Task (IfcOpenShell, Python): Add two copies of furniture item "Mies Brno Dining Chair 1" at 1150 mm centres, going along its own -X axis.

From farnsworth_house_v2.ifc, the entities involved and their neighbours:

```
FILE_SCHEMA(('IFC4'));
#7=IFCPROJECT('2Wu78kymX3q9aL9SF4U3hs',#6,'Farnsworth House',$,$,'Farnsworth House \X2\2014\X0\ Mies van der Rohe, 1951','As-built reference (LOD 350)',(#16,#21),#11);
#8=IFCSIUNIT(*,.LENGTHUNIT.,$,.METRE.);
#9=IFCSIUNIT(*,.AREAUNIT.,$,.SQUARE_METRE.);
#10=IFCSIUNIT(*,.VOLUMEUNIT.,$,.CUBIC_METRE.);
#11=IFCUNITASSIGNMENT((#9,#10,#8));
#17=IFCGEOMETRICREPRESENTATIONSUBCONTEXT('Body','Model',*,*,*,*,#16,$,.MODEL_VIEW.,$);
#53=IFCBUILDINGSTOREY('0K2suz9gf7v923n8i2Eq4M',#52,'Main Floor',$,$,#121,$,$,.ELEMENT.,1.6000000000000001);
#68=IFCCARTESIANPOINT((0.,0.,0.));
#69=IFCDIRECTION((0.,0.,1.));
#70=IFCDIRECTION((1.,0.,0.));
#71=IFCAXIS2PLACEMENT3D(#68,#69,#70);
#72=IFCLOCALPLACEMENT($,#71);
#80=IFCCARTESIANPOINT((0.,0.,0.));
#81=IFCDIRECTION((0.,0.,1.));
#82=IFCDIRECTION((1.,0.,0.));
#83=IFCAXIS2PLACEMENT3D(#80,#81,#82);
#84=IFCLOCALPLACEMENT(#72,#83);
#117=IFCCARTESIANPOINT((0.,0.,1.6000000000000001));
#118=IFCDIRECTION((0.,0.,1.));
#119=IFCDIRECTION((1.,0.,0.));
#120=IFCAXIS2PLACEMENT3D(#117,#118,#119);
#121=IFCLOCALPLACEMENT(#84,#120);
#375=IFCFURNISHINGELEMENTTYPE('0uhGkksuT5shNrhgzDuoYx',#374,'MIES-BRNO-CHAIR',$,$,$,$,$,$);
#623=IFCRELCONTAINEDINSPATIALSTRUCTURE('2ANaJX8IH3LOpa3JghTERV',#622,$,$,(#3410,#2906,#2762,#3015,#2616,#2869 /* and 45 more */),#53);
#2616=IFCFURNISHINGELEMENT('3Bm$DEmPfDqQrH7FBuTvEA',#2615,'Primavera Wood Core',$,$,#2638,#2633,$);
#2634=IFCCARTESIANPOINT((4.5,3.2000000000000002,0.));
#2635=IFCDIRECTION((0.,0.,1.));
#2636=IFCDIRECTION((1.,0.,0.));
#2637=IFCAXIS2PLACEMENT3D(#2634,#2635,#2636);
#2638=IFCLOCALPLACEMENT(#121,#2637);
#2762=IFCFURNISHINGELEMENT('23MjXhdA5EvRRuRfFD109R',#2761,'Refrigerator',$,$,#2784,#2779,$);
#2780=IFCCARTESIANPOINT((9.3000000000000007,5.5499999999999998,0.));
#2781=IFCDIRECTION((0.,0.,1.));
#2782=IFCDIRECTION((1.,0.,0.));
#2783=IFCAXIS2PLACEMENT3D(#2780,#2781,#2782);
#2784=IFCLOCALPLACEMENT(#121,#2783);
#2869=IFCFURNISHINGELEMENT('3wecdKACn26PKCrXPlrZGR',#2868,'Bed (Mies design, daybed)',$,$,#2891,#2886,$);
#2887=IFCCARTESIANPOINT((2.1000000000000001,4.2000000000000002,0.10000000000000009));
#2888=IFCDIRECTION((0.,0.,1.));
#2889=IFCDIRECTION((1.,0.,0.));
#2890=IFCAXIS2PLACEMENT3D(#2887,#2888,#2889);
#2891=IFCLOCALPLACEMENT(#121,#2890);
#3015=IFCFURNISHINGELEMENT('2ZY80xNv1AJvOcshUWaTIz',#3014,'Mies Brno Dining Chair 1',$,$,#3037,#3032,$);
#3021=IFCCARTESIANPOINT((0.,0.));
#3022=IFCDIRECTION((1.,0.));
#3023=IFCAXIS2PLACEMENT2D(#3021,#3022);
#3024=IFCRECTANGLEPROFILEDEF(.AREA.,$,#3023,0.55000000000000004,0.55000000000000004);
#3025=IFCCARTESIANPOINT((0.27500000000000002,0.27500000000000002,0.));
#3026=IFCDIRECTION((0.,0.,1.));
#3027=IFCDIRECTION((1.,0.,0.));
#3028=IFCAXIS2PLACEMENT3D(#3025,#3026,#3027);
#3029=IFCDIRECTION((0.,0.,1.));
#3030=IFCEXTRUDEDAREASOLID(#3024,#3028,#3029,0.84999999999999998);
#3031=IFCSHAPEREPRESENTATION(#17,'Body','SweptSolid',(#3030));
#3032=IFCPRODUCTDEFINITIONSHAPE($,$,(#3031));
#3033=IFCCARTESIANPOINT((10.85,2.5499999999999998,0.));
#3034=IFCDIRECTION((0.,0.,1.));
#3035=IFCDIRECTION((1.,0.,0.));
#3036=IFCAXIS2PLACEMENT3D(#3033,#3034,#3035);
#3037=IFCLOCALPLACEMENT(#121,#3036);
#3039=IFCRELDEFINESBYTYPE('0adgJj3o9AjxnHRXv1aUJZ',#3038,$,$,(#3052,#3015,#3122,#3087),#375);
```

```python
import ifcopenshell
import ifcopenshell.api.geometry
import ifcopenshell.api.root
import ifcopenshell.util.element
import ifcopenshell.util.placement
import ifcopenshell.util.unit

model = ifcopenshell.open("farnsworth_house_v2.ifc")
unit_scale = ifcopenshell.util.unit.calculate_unit_scale(model)


def reuse_history(source, copy):
    """copy_class also copies each property set's owner history, people and application; keep the originals."""
    for rel in copy.IsDefinedBy:
        if rel.is_a("IfcRelDefinesByProperties") and (history := rel.RelatingPropertyDefinition.OwnerHistory):
            rel.RelatingPropertyDefinition.OwnerHistory = source.OwnerHistory
            ifcopenshell.util.element.remove_deep2(model, history)


source = model.by_guid("2ZY80xNv1AJvOcshUWaTIz")
base = ifcopenshell.util.placement.get_local_placement(source.ObjectPlacement)
step = -base[:3, 0] * 1.15 / unit_scale

for i in range(1, 3):
    copy = ifcopenshell.api.root.copy_class(model, product=source)
    copy.Representation = ifcopenshell.util.element.copy_deep(
        model, source.Representation, exclude=["IfcGeometricRepresentationContext", "IfcRepresentationMap"]
    )
    reuse_history(source, copy)
    matrix = base.copy()
    matrix[:3, 3] += i * step
    print("added at", matrix[:3, 3].round(3) + 0.0)
    ifcopenshell.api.geometry.edit_object_placement(model, product=copy, matrix=matrix, is_si=False)

model.write("farnsworth_house_v2_rev.ifc")
```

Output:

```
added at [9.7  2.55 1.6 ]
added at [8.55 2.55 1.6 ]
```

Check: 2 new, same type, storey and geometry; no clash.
